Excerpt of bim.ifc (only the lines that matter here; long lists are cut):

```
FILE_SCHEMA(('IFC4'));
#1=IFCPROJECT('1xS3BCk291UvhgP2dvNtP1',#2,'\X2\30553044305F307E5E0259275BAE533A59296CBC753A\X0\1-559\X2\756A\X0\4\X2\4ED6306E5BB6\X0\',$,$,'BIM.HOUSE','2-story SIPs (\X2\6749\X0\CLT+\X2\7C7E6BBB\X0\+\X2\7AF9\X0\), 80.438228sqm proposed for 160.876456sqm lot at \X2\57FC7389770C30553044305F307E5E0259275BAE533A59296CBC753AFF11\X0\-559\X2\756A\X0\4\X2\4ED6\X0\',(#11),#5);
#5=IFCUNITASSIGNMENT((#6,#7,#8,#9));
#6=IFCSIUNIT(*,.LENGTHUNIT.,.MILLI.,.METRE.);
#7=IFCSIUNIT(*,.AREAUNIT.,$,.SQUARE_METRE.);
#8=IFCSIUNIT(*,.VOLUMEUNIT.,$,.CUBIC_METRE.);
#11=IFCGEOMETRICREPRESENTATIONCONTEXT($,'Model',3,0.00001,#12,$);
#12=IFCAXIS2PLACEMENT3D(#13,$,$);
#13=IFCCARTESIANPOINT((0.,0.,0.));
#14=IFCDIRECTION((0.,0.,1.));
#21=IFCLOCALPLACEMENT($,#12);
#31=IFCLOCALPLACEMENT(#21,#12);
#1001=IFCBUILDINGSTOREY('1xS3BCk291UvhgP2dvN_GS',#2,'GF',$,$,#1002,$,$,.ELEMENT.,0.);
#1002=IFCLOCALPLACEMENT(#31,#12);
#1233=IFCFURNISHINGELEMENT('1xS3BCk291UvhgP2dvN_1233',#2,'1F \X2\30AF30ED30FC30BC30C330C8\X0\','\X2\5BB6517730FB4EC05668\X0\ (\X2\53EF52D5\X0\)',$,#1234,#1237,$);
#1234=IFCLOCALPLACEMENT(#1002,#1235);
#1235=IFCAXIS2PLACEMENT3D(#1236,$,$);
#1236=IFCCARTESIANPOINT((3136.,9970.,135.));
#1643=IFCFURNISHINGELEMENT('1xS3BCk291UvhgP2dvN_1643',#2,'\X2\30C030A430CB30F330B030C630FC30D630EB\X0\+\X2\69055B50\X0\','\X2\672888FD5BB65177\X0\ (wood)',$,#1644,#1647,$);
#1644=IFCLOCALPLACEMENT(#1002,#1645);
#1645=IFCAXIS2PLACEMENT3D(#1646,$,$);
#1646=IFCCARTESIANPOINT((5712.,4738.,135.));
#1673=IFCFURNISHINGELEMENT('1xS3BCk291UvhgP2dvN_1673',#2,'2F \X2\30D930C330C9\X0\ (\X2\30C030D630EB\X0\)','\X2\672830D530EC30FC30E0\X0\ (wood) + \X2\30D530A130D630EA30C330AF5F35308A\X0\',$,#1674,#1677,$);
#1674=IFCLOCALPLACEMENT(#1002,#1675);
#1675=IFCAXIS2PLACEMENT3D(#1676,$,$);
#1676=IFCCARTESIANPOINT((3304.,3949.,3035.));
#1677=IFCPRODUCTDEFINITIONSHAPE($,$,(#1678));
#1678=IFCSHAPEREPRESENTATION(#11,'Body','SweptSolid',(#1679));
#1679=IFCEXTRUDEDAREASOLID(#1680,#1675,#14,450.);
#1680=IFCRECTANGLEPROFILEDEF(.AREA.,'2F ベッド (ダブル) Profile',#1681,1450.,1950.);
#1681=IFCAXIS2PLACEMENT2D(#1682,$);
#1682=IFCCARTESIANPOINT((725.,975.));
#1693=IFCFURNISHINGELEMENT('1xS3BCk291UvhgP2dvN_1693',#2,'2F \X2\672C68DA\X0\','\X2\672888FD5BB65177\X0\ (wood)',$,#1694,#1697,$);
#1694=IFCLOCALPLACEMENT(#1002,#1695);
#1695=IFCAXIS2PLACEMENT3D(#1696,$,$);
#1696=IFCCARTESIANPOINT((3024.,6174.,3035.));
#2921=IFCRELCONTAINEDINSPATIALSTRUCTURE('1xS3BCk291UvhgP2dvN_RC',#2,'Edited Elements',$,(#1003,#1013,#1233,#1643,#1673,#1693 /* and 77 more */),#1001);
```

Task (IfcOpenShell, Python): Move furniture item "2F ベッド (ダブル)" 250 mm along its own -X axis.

```python
import ifcopenshell
import ifcopenshell.api.geometry
import ifcopenshell.util.placement
import ifcopenshell.util.unit

model = ifcopenshell.open("bim.ifc")
unit_scale = ifcopenshell.util.unit.calculate_unit_scale(model)

item = model.by_id(1673)
matrix = ifcopenshell.util.placement.get_local_placement(item.ObjectPlacement)
matrix[:3, 3] -= matrix[:3, 0] * 0.25 / unit_scale
ifcopenshell.api.geometry.edit_object_placement(model, product=item, matrix=matrix, is_si=False)

print(ifcopenshell.util.placement.get_local_placement(item.ObjectPlacement).round(3) + 0.0)

model.write("bim_edited.ifc")
```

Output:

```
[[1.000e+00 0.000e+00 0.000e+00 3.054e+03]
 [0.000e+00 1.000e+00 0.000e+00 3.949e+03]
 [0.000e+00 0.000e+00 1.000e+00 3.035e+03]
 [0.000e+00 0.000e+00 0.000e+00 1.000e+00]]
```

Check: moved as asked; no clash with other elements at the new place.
